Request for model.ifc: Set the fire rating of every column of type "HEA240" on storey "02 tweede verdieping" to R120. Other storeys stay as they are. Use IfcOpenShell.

First a look at what the model holds.

```python
import ifcopenshell
import ifcopenshell.util.element

model = ifcopenshell.open("model.ifc")
print(model.schema)
storey = next(s for s in model.by_type("IfcBuildingStorey") if s.Name == "02 tweede verdieping")
columns = [e for e in ifcopenshell.util.element.get_decomposition(storey) if e.is_a("IfcColumn")]
seen = {}
for e in columns:
    element_type = ifcopenshell.util.element.get_type(e)
    key = (element_type.Name if element_type != e and element_type else None, ifcopenshell.util.element.get_pset(e, "Pset_ColumnCommon", "FireRating"))
    seen[key] = seen.get(key, 0) + 1
for (name, value), count in sorted(seen.items(), key=str):
    print(count, "x", name, "|", value)
```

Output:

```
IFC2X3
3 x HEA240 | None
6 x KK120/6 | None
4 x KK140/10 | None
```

```python
import ifcopenshell
import ifcopenshell.api.pset
import ifcopenshell.util.element

model = ifcopenshell.open("model.ifc")

storey = next(s for s in model.by_type("IfcBuildingStorey") if s.Name == "02 tweede verdieping")
columns = [e for e in ifcopenshell.util.element.get_decomposition(storey) if e.is_a("IfcColumn")]

count = 0
for e in columns:
    element_type = ifcopenshell.util.element.get_type(e)
    if element_type in (None, e) or element_type.Name != "HEA240":
        continue
    found = ifcopenshell.util.element.get_pset(e, "Pset_ColumnCommon", should_inherit=False)
    if found:
        pset = model.by_id(found["id"])
        if len(ifcopenshell.util.element.get_elements_by_pset(pset)) > 1:
            pset = ifcopenshell.api.pset.unshare_pset(model, products=[e], pset=pset)[0]
    else:
        pset = ifcopenshell.api.pset.add_pset(model, product=e, name="Pset_ColumnCommon")
    ifcopenshell.api.pset.edit_pset(model, pset=pset, properties={"FireRating": "R120"})
    count += 1

print(count, "columns updated")

model.write("model_updated.ifc")
```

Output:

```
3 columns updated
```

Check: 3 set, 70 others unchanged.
